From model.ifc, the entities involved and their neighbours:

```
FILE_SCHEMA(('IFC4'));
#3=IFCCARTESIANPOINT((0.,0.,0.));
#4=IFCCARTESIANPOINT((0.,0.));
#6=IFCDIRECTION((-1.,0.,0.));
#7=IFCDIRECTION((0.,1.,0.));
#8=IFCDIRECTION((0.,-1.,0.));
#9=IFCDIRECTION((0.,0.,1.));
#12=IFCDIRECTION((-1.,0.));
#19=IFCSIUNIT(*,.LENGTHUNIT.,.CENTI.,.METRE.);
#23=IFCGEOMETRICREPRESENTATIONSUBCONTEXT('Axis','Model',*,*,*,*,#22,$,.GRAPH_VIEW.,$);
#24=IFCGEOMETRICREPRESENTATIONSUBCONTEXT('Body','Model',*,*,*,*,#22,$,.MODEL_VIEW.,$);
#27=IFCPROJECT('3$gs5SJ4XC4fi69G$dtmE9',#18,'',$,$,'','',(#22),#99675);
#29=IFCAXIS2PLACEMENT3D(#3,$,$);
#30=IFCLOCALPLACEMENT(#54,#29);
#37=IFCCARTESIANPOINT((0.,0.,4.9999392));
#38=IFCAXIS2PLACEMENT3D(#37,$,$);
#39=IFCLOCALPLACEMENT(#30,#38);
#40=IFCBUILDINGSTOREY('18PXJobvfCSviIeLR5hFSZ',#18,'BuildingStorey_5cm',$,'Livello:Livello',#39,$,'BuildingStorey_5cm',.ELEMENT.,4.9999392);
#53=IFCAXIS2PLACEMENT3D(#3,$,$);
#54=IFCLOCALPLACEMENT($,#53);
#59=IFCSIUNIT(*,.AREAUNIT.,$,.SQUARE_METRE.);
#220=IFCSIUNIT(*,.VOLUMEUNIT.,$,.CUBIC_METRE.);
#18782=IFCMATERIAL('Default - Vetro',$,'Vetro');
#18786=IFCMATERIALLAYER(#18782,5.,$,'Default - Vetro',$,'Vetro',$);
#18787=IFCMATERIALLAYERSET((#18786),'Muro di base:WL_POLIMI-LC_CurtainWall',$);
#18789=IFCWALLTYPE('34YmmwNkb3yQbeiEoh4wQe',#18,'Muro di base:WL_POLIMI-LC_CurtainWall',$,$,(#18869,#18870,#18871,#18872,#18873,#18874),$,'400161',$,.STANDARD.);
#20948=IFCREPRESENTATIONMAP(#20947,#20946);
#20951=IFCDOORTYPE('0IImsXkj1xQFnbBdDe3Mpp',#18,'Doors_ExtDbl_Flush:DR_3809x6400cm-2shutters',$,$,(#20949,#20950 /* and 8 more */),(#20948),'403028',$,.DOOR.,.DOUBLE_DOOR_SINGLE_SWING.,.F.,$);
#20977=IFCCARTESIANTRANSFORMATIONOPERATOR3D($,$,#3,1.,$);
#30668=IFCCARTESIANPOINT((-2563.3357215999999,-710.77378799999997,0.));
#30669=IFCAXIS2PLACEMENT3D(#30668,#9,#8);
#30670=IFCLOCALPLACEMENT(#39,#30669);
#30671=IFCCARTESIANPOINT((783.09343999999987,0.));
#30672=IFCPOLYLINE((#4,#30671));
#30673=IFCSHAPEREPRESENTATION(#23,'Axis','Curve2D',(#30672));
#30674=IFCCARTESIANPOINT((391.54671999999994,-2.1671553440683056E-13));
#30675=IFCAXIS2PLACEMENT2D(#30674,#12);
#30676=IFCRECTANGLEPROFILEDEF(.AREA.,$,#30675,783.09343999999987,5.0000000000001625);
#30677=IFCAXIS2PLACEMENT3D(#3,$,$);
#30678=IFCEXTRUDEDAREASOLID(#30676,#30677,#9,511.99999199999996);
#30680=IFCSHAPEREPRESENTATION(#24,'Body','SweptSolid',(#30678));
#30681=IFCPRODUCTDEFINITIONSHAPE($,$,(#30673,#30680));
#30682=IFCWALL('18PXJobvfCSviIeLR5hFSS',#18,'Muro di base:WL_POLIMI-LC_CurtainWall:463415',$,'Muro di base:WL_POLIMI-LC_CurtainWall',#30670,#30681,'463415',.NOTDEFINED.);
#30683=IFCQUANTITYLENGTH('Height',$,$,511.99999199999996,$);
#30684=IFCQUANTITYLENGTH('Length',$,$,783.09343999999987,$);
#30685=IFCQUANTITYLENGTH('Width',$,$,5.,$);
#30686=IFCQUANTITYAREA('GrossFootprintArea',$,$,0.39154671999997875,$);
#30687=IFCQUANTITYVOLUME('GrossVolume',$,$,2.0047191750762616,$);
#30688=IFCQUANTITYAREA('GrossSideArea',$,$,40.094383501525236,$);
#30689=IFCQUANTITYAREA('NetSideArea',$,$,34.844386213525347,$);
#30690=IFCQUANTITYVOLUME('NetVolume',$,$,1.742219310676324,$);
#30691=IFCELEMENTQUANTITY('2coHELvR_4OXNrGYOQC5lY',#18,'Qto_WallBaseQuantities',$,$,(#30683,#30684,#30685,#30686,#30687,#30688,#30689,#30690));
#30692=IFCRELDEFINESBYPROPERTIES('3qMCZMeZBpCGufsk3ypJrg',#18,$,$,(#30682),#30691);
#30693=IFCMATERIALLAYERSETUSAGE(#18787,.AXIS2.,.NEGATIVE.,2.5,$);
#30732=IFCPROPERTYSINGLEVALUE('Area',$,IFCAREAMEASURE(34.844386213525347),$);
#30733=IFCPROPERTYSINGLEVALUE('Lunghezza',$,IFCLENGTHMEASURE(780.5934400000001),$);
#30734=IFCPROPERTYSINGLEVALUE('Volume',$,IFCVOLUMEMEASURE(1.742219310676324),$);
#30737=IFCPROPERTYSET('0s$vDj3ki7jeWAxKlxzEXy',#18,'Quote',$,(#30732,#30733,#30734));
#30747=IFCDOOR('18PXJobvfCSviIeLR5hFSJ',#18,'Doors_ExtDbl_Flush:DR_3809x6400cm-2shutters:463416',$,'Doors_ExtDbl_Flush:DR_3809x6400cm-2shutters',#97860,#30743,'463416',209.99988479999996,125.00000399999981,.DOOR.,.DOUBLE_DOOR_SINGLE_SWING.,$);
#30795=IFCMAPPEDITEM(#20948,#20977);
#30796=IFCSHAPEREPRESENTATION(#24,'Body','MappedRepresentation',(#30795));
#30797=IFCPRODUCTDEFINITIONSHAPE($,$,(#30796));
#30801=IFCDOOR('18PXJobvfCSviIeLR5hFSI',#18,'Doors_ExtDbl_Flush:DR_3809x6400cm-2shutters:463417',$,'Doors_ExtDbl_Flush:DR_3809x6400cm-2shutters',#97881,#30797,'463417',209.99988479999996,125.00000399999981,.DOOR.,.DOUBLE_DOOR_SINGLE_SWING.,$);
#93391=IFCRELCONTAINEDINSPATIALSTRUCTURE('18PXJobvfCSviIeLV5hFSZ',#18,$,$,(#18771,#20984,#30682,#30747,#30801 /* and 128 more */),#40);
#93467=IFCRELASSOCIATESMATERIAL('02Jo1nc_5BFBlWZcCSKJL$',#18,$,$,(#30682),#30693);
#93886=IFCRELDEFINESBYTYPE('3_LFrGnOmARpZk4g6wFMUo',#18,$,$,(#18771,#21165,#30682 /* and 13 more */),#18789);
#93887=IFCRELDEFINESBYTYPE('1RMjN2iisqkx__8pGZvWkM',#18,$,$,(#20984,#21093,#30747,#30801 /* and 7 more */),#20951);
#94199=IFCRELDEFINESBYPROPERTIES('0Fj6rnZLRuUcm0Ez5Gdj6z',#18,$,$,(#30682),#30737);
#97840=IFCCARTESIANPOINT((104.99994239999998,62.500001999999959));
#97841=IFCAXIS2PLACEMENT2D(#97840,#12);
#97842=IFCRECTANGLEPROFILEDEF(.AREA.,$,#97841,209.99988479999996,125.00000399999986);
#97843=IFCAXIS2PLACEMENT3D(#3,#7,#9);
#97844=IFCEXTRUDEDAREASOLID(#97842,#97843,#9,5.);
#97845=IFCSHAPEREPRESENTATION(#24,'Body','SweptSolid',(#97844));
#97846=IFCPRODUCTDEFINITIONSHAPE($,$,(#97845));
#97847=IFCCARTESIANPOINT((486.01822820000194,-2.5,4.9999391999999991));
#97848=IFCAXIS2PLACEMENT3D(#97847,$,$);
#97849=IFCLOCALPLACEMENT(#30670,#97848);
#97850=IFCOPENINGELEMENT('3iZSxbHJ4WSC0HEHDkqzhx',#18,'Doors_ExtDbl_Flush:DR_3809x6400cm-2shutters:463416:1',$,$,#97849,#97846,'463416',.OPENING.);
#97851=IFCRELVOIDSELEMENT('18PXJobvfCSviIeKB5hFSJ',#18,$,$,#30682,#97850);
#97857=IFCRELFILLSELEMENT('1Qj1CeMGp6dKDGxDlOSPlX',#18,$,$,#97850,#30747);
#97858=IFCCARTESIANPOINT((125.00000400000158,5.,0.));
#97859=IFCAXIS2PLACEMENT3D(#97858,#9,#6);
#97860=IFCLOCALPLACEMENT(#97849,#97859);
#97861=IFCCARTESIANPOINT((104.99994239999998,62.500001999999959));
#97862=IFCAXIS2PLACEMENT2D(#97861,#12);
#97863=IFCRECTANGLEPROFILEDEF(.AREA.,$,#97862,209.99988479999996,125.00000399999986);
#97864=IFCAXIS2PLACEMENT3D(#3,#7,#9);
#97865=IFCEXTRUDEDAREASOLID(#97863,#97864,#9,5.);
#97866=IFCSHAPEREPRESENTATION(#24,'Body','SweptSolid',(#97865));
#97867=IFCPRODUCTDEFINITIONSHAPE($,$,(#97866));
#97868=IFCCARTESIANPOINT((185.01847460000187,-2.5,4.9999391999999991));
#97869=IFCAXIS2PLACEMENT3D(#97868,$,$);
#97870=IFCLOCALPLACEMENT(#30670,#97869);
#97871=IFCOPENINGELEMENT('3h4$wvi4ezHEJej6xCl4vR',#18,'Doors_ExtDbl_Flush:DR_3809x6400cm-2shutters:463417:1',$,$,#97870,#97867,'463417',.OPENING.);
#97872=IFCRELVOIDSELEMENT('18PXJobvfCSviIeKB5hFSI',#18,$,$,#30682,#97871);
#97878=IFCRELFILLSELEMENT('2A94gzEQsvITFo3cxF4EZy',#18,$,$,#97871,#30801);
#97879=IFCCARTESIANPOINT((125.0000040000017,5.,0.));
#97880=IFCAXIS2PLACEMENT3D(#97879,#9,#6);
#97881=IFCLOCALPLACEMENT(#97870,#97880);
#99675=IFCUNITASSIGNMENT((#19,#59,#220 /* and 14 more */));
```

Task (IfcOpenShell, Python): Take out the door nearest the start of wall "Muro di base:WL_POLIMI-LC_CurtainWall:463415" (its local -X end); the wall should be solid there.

```python
import ifcopenshell
import ifcopenshell.api.feature
import ifcopenshell.api.pset
import ifcopenshell.api.root
import ifcopenshell.geom
import ifcopenshell.util.element
import ifcopenshell.util.shape
import ifcopenshell.util.unit

model = ifcopenshell.open("model.ifc")
area_scale = ifcopenshell.util.unit.calculate_unit_scale(model, "AREAUNIT")
volume_scale = ifcopenshell.util.unit.calculate_unit_scale(model, "VOLUMEUNIT")
settings = ifcopenshell.geom.settings()


def volume(element):
    """Net volume in cubic metres, openings subtracted."""
    shape = ifcopenshell.geom.create_shape(settings, element)
    return ifcopenshell.util.shape.get_volume(shape.geometry)


door = model.by_guid("18PXJobvfCSviIeLR5hFSI")
opening = door.FillsVoids[0].RelatingOpeningElement
wall = opening.VoidsElements[0].RelatingBuildingElement
before = volume(wall)

ifcopenshell.api.root.remove_product(model, product=door)
ifcopenshell.api.feature.remove_feature(model, feature=opening)

after = volume(wall)
thickness = 0.05  # wall thickness in metres

# Update the wall's stored quantities.
qto = model.by_id(ifcopenshell.util.element.get_pset(wall, "Qto_WallBaseQuantities", should_inherit=False)["id"])
ifcopenshell.api.pset.edit_qto(model, qto=qto, properties={
    "NetSideArea": after / thickness / area_scale,
    "NetVolume": after / volume_scale,
})
pset = model.by_id(ifcopenshell.util.element.get_pset(wall, "Quote", should_inherit=False)["id"])
ifcopenshell.api.pset.edit_pset(model, pset=pset, properties={
    "Area": model.create_entity("IfcAreaMeasure", after / thickness / area_scale),
    "Volume": model.create_entity("IfcVolumeMeasure", after / volume_scale),
})

print(f"wall volume {before:.3f} -> {after:.3f} m3")

model.write("model_rev.ifc")
```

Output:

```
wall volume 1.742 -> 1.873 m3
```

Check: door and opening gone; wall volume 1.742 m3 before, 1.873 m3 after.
